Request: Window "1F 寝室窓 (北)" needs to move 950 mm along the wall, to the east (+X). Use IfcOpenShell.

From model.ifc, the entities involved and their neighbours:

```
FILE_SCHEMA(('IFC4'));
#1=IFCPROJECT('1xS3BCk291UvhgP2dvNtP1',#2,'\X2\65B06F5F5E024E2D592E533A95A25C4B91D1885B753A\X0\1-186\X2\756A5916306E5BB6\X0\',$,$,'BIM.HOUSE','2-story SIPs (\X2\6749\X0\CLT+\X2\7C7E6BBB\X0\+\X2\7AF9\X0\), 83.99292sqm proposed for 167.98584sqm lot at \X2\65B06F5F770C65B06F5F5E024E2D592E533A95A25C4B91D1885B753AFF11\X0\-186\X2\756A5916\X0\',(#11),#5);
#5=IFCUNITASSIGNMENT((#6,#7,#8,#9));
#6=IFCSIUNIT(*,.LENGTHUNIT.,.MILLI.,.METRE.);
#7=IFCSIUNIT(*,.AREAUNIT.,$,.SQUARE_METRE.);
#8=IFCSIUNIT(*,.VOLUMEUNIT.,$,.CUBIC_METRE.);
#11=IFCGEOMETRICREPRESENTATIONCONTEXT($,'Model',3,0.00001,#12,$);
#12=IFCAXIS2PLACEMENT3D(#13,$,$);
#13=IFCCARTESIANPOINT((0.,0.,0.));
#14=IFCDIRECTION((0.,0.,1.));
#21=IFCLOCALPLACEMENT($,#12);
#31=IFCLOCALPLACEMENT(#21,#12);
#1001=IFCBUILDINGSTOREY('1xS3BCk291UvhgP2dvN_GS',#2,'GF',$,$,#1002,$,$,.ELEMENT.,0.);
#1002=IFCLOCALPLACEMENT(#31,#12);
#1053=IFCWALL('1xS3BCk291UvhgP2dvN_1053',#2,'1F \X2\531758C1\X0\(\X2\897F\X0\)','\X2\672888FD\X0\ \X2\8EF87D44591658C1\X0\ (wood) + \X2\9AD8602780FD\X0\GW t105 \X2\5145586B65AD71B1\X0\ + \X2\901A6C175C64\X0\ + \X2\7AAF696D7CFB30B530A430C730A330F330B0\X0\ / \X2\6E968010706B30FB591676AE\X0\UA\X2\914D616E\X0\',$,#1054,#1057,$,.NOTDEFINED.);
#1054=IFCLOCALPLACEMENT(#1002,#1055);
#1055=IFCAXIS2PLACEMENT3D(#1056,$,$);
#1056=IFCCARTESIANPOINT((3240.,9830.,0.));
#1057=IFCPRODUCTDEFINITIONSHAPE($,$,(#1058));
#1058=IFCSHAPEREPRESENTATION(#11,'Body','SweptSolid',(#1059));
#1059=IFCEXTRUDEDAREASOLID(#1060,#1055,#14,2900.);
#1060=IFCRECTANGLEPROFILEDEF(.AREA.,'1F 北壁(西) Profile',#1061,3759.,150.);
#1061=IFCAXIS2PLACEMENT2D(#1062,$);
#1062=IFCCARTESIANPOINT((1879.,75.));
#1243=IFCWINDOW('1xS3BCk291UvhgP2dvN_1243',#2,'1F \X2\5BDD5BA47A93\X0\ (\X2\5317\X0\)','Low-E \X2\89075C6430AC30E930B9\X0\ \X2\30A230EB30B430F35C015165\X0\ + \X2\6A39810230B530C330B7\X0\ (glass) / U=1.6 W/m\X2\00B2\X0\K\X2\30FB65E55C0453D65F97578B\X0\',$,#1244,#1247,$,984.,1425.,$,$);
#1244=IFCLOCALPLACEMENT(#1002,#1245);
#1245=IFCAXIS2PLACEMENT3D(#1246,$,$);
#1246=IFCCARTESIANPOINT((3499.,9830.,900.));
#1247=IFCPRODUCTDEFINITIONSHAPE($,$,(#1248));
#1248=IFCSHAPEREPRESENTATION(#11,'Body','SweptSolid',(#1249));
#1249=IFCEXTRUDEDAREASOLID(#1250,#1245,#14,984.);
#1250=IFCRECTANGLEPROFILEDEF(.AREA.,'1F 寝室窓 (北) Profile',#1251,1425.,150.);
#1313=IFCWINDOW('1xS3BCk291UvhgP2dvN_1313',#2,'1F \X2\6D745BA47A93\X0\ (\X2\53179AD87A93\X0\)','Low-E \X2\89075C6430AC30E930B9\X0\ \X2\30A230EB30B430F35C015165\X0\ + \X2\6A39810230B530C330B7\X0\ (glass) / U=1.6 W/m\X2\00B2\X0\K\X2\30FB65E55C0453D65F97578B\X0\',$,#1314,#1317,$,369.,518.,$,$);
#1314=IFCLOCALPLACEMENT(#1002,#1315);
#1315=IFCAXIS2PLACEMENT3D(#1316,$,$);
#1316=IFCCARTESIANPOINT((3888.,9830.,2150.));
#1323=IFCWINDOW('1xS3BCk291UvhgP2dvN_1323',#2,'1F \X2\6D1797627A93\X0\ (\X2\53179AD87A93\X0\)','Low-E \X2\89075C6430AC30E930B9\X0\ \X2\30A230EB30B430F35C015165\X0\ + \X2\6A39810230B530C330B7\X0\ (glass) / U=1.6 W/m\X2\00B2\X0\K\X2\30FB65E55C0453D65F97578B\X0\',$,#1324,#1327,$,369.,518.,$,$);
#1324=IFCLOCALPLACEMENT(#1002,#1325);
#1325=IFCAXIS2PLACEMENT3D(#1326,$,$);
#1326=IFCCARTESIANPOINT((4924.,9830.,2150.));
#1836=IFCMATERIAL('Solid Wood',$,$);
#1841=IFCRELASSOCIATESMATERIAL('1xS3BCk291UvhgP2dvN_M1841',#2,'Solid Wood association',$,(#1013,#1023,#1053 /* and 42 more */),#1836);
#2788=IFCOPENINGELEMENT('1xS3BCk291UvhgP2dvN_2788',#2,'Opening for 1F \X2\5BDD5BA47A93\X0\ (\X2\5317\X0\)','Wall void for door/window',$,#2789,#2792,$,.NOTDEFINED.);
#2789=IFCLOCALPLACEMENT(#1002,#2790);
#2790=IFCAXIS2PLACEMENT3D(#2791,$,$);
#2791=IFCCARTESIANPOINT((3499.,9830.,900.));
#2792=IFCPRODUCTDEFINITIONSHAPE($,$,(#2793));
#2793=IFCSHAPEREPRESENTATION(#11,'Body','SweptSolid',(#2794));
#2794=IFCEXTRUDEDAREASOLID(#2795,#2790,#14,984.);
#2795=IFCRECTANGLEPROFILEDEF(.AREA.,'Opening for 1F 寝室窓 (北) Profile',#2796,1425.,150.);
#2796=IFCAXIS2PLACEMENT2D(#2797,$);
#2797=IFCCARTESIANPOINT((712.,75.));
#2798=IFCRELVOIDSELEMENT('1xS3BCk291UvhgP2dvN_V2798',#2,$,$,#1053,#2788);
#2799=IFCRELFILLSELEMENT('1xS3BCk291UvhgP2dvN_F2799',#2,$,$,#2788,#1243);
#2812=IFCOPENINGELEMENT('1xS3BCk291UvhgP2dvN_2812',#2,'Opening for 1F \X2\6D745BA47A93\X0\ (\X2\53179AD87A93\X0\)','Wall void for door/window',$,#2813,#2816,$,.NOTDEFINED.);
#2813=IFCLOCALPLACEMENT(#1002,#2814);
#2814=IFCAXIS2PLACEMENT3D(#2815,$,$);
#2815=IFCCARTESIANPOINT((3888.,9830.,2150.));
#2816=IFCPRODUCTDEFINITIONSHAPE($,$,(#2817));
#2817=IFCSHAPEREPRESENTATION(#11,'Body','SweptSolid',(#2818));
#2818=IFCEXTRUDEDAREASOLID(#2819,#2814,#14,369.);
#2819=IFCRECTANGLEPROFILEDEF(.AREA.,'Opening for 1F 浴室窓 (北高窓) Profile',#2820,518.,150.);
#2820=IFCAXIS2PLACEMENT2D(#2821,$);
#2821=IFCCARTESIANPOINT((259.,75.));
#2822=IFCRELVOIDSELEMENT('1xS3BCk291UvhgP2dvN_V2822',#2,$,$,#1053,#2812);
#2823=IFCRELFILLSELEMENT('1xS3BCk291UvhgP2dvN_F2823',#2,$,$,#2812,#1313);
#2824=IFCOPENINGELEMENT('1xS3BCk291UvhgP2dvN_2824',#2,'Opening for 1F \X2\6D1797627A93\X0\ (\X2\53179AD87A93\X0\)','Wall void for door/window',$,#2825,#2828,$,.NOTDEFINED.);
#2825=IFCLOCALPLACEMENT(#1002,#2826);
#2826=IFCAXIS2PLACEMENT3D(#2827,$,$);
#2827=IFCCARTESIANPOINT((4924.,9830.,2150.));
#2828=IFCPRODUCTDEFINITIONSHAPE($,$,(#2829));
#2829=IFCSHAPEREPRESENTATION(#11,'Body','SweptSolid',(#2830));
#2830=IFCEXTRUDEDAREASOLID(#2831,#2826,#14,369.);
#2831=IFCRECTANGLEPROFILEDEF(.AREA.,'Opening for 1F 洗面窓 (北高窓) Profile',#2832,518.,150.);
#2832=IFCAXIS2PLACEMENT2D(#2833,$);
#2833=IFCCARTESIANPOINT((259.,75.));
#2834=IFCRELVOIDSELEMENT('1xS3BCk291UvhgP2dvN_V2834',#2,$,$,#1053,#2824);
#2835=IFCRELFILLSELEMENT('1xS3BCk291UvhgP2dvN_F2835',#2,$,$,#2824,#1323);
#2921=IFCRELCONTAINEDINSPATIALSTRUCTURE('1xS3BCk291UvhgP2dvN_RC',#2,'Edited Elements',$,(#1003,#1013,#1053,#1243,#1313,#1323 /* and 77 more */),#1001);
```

```python
import ifcopenshell
import ifcopenshell.api.geometry
import ifcopenshell.util.placement

model = ifcopenshell.open("model.ifc")

window = model.by_guid("1xS3BCk291UvhgP2dvN_1243")
opening = window.FillsVoids[0].RelatingOpeningElement
wall = opening.VoidsElements[0].RelatingBuildingElement

wall_matrix = ifcopenshell.util.placement.get_local_placement(wall.ObjectPlacement)
shift = wall_matrix[:3, 0] * 950.0
before = ifcopenshell.util.placement.get_local_placement(window.ObjectPlacement)[:3, 3].copy()

# The window is not placed relative to its opening, so move both.
for product in (opening, window):
    matrix = ifcopenshell.util.placement.get_local_placement(product.ObjectPlacement)
    matrix[:3, 3] += shift
    ifcopenshell.api.geometry.edit_object_placement(model, product=product, matrix=matrix, is_si=False)

after = ifcopenshell.util.placement.get_local_placement(window.ObjectPlacement)[:3, 3]
print("window moved by", (after - before).round(3) + 0.0)

model.write("model_edited.ifc")
```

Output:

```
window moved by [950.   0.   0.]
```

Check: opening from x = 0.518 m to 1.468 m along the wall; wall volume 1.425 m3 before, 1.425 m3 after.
